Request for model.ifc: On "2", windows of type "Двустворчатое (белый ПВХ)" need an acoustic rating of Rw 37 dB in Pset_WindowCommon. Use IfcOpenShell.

First a look at what the model holds.

```python
import ifcopenshell
import ifcopenshell.util.element

model = ifcopenshell.open("model.ifc")
print(model.schema)
storey = next(s for s in model.by_type("IfcBuildingStorey") if s.Name == "2")
windows = [e for e in ifcopenshell.util.element.get_decomposition(storey) if e.is_a("IfcWindow")]
seen = {}
for e in windows:
    element_type = ifcopenshell.util.element.get_type(e)
    key = (element_type.Name if element_type != e and element_type else None, ifcopenshell.util.element.get_pset(e, "Pset_WindowCommon", "AcousticRating"))
    seen[key] = seen.get(key, 0) + 1
for (name, value), count in sorted(seen.items(), key=str):
    print(count, "x", name, "|", value)
```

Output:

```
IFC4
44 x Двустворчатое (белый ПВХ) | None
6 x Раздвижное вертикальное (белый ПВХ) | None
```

```python
import ifcopenshell
import ifcopenshell.api.pset
import ifcopenshell.util.element

model = ifcopenshell.open("model.ifc")

storey = next(s for s in model.by_type("IfcBuildingStorey") if s.Name == "2")
windows = [e for e in ifcopenshell.util.element.get_decomposition(storey) if e.is_a("IfcWindow")]

count = 0
for e in windows:
    element_type = ifcopenshell.util.element.get_type(e)
    if element_type in (None, e) or element_type.Name != "Двустворчатое (белый ПВХ)":
        continue
    # add_pset returns the element's existing set when there is one.
    pset = ifcopenshell.api.pset.add_pset(model, product=e, name="Pset_WindowCommon")
    ifcopenshell.api.pset.edit_pset(model, pset=pset, properties={"AcousticRating": "Rw 37 dB"})
    count += 1

print(count, "windows updated")

model.write("model_updated.ifc")
```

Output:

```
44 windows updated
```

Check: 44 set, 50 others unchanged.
